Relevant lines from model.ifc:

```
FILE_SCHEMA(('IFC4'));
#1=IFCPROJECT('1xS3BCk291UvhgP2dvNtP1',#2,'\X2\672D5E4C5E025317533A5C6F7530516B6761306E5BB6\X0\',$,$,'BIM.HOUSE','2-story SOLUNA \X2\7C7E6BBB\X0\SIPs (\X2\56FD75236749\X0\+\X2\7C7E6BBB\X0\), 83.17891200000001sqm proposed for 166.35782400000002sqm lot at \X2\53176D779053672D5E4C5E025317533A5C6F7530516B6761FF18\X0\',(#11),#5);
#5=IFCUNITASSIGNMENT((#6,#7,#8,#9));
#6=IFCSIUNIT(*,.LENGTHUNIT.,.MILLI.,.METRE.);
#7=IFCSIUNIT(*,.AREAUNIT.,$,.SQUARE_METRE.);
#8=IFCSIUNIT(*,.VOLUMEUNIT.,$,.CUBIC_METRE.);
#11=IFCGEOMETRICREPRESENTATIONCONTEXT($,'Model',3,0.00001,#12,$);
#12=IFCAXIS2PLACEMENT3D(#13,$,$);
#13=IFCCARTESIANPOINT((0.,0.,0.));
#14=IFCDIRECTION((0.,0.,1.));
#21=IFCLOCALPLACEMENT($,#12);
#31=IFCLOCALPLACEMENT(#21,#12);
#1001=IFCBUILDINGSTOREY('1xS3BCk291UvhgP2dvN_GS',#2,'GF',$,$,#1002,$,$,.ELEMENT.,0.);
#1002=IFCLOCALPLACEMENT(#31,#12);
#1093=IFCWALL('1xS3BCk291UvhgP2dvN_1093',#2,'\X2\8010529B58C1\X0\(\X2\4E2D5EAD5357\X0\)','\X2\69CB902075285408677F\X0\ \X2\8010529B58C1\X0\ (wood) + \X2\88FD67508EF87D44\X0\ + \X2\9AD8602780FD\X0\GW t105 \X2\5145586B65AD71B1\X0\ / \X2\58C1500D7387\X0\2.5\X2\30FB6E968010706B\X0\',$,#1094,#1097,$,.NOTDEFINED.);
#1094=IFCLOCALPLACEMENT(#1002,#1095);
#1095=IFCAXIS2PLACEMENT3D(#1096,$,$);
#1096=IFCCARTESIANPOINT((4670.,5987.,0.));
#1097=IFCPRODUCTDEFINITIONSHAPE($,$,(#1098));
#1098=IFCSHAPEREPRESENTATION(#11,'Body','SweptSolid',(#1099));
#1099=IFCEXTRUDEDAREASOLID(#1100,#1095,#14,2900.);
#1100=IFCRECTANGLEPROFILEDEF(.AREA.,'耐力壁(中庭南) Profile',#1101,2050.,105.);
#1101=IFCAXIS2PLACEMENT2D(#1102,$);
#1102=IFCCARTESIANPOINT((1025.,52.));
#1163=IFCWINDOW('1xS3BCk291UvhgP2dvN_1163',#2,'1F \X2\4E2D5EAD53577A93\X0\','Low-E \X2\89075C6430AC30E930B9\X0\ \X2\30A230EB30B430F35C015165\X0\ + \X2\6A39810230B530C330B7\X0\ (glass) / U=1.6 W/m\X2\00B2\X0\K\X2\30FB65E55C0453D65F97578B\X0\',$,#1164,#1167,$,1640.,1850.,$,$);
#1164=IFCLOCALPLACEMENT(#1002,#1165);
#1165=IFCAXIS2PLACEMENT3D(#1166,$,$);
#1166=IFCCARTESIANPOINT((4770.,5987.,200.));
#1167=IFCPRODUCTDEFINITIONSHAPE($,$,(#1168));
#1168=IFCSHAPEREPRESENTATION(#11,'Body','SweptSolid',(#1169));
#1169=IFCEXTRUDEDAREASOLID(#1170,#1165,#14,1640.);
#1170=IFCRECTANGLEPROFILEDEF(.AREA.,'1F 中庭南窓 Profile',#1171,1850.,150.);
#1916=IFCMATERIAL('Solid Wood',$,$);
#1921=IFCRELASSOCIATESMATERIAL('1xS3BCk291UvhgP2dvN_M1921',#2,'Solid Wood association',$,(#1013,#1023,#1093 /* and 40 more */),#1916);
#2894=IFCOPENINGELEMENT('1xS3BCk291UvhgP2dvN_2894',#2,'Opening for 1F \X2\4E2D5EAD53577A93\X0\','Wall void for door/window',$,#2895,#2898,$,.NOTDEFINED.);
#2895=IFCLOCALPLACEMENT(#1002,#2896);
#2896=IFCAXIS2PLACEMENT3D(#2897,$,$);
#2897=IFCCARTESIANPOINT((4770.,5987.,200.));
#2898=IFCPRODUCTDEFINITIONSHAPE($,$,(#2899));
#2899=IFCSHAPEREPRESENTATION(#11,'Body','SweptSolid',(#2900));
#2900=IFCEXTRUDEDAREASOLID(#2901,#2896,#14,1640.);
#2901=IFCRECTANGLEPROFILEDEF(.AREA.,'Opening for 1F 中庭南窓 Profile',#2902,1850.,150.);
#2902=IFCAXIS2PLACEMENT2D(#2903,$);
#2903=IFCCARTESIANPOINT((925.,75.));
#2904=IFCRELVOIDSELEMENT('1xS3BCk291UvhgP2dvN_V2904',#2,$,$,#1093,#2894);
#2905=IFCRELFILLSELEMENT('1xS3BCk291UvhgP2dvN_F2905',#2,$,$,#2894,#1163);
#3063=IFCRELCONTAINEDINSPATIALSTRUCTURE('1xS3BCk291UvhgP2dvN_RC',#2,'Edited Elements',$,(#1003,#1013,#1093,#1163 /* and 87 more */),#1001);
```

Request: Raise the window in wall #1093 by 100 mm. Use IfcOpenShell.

```python
import numpy as np
import ifcopenshell
import ifcopenshell.api.geometry
import ifcopenshell.util.placement
import ifcopenshell.util.unit

model = ifcopenshell.open("model.ifc")
unit_scale = ifcopenshell.util.unit.calculate_unit_scale(model)

window = model.by_guid("1xS3BCk291UvhgP2dvN_1163")
opening = window.FillsVoids[0].RelatingOpeningElement
dz = 100.0

shift = np.array([0.0, 0.0, dz])
# The window is not placed relative to its opening, so move both.
for product in (opening, window):
    matrix = ifcopenshell.util.placement.get_local_placement(product.ObjectPlacement)
    matrix[:3, 3] += shift
    ifcopenshell.api.geometry.edit_object_placement(model, product=product, matrix=matrix, is_si=False)

print(f"moved by {dz * unit_scale:+.3f} m")

model.write("model_v2.ifc")
```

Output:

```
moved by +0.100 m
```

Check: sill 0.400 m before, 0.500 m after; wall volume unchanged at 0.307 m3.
